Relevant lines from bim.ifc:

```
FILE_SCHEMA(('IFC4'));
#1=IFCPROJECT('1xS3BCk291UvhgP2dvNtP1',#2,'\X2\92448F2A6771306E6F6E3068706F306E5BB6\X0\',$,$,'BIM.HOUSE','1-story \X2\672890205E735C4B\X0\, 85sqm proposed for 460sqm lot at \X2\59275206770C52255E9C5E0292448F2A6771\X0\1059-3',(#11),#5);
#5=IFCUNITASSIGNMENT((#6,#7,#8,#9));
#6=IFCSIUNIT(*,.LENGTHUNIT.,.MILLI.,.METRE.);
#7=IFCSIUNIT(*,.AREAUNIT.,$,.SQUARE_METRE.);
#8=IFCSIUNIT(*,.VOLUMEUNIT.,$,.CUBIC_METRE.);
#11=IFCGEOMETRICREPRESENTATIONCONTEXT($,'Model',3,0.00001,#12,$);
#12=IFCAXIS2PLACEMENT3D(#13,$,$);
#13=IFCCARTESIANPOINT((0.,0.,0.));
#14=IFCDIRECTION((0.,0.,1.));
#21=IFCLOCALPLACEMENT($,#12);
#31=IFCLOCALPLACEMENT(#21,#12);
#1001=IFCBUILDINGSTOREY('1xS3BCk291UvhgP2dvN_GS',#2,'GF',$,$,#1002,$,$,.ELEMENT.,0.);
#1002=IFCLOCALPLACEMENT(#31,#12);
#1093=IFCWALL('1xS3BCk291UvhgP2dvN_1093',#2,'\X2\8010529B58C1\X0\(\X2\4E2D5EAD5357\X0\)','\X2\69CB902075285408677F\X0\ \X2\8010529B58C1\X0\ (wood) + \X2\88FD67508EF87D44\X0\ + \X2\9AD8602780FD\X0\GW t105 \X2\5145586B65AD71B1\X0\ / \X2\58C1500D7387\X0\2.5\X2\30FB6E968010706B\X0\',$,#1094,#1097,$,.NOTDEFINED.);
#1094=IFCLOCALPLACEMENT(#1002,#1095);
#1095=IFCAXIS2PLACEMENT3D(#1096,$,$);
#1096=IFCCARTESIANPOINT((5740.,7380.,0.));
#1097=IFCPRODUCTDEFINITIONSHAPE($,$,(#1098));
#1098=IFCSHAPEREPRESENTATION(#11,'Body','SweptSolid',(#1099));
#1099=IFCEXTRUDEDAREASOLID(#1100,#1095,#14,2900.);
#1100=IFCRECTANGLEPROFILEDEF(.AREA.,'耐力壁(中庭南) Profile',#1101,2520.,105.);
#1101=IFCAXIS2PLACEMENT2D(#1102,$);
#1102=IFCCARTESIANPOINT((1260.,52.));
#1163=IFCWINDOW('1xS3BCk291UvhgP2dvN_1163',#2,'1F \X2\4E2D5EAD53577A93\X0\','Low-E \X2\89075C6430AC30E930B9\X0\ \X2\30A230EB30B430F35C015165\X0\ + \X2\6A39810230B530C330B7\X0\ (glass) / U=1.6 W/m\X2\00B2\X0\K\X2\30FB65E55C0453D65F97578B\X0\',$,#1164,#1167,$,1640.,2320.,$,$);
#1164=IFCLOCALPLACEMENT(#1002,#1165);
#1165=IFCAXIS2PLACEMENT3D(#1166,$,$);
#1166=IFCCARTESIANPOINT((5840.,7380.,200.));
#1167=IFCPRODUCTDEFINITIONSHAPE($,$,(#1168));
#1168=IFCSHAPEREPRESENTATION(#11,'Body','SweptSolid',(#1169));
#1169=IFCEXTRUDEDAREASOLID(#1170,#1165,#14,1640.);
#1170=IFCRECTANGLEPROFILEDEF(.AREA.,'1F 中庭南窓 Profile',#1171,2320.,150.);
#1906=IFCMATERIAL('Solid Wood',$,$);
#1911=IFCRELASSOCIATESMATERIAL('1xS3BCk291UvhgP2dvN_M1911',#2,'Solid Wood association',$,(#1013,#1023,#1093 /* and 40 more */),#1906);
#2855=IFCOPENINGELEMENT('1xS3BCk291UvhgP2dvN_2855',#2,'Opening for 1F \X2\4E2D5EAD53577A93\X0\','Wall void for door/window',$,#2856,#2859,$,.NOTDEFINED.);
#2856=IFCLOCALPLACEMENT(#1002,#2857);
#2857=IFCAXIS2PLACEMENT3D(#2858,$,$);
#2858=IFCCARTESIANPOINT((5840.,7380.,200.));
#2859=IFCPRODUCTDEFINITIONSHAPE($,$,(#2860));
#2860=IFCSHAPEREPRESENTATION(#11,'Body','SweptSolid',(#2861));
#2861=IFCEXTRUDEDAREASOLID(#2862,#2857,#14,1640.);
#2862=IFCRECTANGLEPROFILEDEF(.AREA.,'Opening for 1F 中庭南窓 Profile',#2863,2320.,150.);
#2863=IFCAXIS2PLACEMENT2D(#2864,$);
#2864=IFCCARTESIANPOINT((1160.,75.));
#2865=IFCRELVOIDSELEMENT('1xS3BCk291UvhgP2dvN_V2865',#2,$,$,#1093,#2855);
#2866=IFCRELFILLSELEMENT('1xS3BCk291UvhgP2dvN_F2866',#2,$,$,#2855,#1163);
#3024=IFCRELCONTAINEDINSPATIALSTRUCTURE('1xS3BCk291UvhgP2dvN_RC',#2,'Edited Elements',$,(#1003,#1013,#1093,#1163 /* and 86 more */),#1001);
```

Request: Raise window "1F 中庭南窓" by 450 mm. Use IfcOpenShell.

```python
import numpy as np
import ifcopenshell
import ifcopenshell.api.geometry
import ifcopenshell.util.placement
import ifcopenshell.util.unit

model = ifcopenshell.open("bim.ifc")
unit_scale = ifcopenshell.util.unit.calculate_unit_scale(model)

window = model.by_guid("1xS3BCk291UvhgP2dvN_1163")
opening = window.FillsVoids[0].RelatingOpeningElement
dz = 450.0

shift = np.array([0.0, 0.0, dz])
# The window is not placed relative to its opening, so move both.
for product in (opening, window):
    matrix = ifcopenshell.util.placement.get_local_placement(product.ObjectPlacement)
    matrix[:3, 3] += shift
    ifcopenshell.api.geometry.edit_object_placement(model, product=product, matrix=matrix, is_si=False)

print(f"moved by {dz * unit_scale:+.3f} m")

model.write("bim_rev.ifc")
```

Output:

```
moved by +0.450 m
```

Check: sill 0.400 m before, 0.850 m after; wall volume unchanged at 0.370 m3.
